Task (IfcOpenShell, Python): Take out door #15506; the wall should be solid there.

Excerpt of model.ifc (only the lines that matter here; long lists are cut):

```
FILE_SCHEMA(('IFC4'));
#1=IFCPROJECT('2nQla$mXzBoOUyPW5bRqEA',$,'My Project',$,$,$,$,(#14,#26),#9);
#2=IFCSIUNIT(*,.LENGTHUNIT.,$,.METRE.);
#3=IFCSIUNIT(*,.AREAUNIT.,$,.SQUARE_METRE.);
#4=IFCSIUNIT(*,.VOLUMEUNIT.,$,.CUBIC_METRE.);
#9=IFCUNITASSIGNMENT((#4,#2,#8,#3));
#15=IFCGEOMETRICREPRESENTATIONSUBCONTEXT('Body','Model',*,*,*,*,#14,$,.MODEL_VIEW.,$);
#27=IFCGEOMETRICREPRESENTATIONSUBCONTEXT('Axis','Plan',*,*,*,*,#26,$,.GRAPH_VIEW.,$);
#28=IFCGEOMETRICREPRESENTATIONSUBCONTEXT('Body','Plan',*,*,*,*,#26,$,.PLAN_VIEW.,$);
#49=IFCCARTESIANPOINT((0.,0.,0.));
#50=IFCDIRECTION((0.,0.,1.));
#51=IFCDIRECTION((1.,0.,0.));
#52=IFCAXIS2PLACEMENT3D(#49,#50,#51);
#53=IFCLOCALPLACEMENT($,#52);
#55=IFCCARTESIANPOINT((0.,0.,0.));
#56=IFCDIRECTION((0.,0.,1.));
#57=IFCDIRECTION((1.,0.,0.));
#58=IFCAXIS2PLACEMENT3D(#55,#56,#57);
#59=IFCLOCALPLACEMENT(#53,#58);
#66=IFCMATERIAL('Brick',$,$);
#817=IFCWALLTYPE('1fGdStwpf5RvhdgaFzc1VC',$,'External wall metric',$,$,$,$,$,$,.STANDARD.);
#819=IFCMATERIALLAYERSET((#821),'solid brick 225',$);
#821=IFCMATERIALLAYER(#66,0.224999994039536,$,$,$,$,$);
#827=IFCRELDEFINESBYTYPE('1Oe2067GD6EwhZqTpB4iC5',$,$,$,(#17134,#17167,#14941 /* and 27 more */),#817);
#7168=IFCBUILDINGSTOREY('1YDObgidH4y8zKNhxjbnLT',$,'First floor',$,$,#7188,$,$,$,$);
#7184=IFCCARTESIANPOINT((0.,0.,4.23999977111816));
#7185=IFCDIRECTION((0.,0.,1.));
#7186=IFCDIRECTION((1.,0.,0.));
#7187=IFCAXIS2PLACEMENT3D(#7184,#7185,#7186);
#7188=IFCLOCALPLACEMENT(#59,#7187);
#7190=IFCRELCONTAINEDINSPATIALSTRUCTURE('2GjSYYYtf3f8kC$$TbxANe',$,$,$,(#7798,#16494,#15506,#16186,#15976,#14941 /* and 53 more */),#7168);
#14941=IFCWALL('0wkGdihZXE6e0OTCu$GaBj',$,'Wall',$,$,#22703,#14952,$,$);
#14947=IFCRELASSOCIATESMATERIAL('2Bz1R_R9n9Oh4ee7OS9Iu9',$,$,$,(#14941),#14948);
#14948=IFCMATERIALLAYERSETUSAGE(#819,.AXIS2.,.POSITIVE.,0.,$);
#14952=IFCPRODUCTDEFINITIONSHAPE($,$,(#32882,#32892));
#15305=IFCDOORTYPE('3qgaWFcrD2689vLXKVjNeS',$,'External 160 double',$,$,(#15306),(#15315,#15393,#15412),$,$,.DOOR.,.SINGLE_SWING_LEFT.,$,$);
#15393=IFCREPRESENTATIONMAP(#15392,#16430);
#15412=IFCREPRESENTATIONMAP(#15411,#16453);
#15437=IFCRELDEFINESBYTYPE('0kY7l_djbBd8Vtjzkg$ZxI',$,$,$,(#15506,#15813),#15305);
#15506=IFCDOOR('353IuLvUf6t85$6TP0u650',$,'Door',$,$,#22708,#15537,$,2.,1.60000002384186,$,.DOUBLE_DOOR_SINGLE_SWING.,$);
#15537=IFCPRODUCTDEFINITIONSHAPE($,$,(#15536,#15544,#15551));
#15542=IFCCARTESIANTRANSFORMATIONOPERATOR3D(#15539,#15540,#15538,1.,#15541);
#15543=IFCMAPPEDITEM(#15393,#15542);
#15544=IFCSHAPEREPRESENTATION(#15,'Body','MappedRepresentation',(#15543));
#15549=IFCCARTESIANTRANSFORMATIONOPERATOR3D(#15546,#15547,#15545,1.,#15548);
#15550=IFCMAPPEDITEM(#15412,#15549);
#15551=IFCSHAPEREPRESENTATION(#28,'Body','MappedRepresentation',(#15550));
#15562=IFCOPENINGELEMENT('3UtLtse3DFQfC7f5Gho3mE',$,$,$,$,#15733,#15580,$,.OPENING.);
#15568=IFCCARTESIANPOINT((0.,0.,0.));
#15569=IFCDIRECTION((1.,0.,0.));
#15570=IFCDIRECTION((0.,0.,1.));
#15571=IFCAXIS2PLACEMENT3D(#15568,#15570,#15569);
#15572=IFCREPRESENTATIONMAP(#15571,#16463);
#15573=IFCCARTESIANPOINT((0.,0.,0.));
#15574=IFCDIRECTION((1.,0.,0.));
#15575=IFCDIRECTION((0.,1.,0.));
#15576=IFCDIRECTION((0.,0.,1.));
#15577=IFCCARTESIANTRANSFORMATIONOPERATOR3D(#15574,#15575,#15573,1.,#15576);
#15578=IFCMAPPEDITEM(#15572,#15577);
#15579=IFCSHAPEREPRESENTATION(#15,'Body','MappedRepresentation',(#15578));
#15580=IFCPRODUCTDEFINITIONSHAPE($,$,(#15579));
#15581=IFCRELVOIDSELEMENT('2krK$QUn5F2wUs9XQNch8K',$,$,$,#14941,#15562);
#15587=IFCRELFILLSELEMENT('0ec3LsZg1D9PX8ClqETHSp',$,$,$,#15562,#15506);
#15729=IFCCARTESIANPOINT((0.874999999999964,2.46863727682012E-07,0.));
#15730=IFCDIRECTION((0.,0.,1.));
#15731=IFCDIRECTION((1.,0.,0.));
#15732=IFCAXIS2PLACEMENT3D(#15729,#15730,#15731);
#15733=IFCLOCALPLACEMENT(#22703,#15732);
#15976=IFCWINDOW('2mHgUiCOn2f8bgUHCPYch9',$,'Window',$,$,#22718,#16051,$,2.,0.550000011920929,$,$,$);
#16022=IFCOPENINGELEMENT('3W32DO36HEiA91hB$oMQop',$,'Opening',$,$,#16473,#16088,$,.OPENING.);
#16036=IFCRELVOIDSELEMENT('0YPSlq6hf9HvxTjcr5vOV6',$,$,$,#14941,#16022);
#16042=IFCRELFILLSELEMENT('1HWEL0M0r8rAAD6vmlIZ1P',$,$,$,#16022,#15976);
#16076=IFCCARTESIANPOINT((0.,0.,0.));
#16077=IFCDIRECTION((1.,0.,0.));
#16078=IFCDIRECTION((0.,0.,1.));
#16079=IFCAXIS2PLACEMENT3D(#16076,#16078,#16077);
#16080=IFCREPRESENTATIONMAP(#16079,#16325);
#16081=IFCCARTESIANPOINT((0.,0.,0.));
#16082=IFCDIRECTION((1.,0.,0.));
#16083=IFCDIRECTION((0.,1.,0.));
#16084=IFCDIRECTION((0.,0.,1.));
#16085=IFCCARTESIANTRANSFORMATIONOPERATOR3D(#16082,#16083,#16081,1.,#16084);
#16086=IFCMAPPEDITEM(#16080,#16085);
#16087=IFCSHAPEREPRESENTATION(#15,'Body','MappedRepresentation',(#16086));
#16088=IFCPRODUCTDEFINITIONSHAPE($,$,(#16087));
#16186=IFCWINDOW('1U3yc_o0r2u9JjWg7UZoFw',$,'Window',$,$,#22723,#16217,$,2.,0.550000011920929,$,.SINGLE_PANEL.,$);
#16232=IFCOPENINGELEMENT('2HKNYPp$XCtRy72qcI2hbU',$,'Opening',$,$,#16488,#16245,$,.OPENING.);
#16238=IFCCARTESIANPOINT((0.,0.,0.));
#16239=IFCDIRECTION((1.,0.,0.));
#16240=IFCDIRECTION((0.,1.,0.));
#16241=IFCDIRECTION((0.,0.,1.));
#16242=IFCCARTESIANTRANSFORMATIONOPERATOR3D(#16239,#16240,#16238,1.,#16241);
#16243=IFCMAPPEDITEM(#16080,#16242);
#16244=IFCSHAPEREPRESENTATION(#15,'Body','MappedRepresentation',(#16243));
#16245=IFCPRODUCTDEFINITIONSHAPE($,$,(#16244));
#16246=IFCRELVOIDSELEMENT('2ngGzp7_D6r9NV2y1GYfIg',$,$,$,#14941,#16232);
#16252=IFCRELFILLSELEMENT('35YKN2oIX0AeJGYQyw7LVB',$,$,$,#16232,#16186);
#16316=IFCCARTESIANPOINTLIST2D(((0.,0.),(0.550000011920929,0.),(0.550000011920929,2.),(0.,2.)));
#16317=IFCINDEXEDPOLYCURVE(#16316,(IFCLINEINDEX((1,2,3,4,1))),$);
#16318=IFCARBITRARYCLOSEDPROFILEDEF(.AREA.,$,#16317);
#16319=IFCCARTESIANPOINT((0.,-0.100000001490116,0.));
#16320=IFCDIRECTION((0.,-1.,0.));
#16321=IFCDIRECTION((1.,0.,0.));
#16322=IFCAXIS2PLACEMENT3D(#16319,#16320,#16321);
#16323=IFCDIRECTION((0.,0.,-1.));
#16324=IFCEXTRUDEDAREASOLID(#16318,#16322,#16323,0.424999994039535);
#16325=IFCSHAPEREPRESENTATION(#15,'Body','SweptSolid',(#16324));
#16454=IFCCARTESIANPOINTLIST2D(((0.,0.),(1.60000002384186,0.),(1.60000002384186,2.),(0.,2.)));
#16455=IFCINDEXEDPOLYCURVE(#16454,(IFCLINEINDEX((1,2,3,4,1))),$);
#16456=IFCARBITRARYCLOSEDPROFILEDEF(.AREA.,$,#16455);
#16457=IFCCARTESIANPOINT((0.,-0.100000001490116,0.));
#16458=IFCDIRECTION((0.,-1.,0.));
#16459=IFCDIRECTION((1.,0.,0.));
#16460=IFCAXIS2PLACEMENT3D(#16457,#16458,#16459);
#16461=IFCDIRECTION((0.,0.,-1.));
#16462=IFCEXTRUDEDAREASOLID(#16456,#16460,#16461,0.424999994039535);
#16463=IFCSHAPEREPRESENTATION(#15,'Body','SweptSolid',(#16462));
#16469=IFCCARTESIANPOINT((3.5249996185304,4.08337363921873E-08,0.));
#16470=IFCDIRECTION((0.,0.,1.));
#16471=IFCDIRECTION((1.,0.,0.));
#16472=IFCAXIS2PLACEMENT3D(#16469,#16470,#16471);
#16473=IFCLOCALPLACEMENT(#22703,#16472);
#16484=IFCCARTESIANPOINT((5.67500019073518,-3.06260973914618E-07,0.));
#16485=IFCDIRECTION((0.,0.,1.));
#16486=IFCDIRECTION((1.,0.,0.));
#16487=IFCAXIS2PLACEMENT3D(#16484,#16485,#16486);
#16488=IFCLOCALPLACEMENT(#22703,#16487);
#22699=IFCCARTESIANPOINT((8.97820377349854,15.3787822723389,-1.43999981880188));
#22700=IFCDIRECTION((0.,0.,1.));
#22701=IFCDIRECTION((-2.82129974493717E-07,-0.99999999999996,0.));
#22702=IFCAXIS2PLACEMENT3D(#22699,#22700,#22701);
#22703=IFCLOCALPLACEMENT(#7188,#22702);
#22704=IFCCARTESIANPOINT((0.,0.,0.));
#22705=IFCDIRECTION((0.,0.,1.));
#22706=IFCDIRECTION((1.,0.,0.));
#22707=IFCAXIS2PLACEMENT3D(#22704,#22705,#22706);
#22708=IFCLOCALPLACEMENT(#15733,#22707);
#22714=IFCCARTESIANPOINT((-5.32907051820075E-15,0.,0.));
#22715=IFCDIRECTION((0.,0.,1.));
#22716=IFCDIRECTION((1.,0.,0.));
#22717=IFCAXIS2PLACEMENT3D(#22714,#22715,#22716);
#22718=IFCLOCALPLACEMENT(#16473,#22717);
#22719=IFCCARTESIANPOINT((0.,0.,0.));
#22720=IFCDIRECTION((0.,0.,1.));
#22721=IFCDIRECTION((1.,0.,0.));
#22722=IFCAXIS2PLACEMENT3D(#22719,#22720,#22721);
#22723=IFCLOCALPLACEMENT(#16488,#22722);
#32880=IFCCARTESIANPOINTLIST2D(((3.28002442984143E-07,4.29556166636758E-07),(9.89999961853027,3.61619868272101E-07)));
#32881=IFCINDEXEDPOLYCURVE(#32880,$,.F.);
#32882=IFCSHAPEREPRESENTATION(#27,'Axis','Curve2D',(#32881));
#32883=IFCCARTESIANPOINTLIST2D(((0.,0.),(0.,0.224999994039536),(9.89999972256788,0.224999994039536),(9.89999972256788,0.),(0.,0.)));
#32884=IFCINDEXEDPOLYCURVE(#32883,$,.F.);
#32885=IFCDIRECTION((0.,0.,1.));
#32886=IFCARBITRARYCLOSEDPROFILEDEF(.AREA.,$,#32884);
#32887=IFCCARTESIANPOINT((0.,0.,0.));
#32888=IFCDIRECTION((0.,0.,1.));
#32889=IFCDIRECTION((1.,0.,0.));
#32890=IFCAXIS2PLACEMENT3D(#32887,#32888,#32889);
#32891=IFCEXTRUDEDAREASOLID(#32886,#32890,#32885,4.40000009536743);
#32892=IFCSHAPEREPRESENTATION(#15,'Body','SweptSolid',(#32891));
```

```python
import ifcopenshell
import ifcopenshell.api.feature
import ifcopenshell.api.root
import ifcopenshell.geom
import ifcopenshell.util.shape

model = ifcopenshell.open("model.ifc")
settings = ifcopenshell.geom.settings()


def volume(element):
    """Net volume in cubic metres, openings subtracted."""
    shape = ifcopenshell.geom.create_shape(settings, element)
    return ifcopenshell.util.shape.get_volume(shape.geometry)


door = model.by_guid("353IuLvUf6t85$6TP0u650")
opening = door.FillsVoids[0].RelatingOpeningElement
wall = opening.VoidsElements[0].RelatingBuildingElement
before = volume(wall)

ifcopenshell.api.root.remove_product(model, product=door)
ifcopenshell.api.feature.remove_feature(model, feature=opening)

after = volume(wall)

print(f"wall volume {before:.3f} -> {after:.3f} m3")

model.write("model_edited.ifc")
```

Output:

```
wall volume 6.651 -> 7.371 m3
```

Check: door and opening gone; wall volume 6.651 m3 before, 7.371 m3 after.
